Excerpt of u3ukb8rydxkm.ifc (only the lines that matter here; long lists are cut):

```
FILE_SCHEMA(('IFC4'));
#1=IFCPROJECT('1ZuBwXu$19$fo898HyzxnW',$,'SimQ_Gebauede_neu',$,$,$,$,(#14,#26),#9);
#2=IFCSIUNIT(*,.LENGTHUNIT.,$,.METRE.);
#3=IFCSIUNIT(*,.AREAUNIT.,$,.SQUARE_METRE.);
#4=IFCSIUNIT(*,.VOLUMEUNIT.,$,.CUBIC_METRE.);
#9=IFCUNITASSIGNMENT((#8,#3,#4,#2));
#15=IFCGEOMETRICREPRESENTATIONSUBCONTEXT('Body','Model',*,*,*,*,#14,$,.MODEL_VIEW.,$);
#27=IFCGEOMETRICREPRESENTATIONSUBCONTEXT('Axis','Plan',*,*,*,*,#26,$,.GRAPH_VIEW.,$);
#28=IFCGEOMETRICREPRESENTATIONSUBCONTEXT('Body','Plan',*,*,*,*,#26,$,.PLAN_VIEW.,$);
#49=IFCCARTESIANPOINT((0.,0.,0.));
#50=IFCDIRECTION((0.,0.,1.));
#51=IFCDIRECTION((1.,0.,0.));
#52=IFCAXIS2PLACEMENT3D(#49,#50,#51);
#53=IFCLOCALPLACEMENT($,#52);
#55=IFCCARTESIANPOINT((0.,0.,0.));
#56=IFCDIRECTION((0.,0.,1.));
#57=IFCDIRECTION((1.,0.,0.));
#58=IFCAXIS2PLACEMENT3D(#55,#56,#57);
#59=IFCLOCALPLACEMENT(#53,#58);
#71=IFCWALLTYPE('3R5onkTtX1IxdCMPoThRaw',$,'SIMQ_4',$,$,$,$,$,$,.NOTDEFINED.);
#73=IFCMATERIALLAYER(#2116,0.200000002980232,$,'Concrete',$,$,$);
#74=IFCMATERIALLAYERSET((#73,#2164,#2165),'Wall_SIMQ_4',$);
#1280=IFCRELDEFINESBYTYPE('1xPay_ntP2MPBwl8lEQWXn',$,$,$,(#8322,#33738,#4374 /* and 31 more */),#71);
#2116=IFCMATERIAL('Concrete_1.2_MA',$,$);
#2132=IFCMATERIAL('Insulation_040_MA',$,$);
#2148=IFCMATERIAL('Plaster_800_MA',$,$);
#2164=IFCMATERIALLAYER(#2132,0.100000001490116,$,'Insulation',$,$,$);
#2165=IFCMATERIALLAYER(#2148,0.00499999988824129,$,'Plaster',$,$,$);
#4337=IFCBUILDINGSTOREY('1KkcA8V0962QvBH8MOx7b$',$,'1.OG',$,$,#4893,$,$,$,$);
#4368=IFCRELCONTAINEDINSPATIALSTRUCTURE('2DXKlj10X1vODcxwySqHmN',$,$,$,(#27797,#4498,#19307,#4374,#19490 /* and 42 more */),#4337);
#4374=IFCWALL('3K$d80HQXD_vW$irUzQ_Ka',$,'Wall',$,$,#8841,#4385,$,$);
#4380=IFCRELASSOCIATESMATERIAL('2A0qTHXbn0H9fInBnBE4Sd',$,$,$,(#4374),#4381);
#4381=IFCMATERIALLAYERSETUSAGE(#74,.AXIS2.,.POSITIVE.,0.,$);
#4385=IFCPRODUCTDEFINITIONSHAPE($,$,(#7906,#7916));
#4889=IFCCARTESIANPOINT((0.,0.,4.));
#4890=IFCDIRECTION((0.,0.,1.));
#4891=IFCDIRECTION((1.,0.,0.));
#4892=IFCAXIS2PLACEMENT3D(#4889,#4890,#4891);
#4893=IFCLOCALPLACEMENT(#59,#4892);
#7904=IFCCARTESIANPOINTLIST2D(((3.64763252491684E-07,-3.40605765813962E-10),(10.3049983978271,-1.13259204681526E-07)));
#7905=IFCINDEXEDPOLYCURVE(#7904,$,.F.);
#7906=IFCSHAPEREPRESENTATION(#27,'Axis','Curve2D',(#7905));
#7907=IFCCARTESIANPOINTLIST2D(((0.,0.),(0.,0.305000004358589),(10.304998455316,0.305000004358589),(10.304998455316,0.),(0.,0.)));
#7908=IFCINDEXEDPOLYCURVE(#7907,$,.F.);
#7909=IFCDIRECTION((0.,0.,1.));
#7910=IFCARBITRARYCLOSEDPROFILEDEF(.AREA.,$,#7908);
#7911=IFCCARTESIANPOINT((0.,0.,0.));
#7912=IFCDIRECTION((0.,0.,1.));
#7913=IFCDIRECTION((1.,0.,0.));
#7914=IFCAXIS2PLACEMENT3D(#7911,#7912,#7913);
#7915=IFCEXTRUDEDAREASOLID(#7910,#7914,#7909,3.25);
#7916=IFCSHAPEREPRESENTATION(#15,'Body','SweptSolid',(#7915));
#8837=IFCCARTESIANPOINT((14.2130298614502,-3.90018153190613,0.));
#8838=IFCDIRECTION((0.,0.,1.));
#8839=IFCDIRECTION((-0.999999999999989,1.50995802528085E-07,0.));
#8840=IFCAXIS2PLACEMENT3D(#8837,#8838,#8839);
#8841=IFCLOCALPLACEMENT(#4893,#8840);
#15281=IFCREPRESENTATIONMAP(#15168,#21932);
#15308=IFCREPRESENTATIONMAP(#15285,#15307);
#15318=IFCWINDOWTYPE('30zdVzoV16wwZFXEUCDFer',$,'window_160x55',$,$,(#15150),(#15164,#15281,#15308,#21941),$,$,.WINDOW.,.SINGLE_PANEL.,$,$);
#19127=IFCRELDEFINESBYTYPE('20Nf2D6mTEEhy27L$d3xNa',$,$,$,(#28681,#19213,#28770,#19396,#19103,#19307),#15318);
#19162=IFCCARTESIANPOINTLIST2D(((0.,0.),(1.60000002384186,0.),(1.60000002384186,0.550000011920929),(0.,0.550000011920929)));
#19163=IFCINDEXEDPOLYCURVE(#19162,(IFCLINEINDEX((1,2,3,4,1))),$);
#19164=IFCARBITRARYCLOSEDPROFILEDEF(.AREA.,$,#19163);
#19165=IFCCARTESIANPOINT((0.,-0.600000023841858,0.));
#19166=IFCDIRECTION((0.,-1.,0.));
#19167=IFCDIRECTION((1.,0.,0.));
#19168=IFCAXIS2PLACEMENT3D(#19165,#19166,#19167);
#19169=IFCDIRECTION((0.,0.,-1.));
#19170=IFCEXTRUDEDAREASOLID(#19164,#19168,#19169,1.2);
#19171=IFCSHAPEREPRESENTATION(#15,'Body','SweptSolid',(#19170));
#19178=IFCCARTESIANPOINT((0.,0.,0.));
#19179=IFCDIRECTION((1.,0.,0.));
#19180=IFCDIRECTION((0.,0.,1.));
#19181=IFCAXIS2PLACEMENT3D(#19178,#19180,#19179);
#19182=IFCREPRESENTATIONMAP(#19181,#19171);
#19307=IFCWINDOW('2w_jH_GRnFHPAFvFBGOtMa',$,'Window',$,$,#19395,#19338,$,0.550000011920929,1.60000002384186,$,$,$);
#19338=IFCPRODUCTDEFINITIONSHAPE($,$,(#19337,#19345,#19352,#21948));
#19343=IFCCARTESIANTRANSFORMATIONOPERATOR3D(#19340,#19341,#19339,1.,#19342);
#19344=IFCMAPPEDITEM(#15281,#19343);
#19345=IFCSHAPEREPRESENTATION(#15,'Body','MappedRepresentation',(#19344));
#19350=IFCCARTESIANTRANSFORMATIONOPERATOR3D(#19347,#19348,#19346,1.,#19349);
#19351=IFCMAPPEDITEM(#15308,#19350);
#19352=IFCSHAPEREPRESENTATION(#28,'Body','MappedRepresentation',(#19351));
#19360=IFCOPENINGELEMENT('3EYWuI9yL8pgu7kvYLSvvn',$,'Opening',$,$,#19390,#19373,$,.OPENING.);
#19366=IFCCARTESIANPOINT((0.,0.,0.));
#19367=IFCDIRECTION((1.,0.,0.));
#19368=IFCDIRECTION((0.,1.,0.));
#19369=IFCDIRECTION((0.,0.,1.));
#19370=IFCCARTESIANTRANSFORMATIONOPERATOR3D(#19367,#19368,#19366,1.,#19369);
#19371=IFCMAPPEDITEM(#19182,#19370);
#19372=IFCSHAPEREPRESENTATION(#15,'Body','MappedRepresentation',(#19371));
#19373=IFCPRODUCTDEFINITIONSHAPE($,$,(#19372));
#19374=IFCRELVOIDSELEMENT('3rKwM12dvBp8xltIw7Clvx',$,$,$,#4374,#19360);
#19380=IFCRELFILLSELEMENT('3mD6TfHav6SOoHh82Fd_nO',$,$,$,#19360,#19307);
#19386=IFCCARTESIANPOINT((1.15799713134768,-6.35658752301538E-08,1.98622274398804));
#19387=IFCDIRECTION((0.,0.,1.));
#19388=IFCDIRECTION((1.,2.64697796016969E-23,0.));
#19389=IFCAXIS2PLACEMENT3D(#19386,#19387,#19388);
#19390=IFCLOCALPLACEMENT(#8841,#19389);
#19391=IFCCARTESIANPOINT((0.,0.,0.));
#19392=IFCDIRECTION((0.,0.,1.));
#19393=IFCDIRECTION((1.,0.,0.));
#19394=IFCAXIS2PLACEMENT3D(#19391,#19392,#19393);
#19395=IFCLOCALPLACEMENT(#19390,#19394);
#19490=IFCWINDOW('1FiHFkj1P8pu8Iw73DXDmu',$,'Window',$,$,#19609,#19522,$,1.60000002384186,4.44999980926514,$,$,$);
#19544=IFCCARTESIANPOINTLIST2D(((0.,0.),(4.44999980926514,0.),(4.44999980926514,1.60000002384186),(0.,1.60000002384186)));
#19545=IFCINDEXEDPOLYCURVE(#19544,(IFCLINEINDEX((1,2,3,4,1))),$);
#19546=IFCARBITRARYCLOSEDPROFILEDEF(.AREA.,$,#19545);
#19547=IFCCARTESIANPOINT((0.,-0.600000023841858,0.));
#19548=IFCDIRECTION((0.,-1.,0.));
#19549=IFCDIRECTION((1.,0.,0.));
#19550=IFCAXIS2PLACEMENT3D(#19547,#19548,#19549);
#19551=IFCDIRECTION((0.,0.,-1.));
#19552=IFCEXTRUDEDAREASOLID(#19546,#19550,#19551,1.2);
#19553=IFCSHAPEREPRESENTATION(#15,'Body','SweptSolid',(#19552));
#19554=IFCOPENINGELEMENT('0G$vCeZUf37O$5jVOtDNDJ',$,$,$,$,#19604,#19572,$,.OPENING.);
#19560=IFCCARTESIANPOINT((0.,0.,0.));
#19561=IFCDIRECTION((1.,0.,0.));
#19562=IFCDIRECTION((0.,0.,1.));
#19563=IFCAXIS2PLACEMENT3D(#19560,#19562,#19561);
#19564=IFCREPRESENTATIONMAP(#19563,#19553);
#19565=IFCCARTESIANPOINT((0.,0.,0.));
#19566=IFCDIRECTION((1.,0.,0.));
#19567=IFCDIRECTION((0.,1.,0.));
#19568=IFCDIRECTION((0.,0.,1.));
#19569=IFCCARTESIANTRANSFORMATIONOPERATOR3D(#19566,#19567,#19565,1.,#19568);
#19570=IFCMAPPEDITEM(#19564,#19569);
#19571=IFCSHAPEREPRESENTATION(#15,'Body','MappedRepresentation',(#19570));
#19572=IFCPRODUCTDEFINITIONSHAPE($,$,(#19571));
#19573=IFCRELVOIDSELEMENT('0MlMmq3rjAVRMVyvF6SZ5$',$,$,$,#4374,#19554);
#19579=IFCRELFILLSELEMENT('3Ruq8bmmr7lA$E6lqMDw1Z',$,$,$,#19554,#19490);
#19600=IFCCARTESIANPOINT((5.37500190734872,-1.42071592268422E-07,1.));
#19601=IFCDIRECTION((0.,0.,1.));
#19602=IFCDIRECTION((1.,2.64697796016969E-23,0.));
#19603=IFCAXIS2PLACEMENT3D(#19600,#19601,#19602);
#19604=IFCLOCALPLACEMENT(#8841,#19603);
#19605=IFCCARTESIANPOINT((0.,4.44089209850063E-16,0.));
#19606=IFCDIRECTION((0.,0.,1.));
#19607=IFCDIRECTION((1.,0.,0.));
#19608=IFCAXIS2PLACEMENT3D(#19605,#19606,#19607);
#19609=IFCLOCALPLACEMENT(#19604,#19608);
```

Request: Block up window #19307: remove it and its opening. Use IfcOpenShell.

```python
import ifcopenshell
import ifcopenshell.api.feature
import ifcopenshell.api.root
import ifcopenshell.geom
import ifcopenshell.util.shape

model = ifcopenshell.open("u3ukb8rydxkm.ifc")
settings = ifcopenshell.geom.settings()


def volume(element):
    """Net volume in cubic metres, openings subtracted."""
    shape = ifcopenshell.geom.create_shape(settings, element)
    return ifcopenshell.util.shape.get_volume(shape.geometry)


window = model.by_guid("2w_jH_GRnFHPAFvFBGOtMa")
opening = window.FillsVoids[0].RelatingOpeningElement
wall = opening.VoidsElements[0].RelatingBuildingElement
before = volume(wall)

ifcopenshell.api.root.remove_product(model, product=window)
ifcopenshell.api.feature.remove_feature(model, feature=opening)

after = volume(wall)

print(f"wall volume {before:.3f} -> {after:.3f} m3")

model.write("u3ukb8rydxkm_edited.ifc")
```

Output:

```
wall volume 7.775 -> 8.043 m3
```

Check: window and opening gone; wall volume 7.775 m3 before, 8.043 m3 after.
